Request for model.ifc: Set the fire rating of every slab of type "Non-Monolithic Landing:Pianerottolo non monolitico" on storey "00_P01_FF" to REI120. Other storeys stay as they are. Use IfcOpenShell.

First a look at what the model holds.

```python
import ifcopenshell
import ifcopenshell.util.element

model = ifcopenshell.open("model.ifc")
print(model.schema)
storey = next(s for s in model.by_type("IfcBuildingStorey") if s.Name == "00_P01_FF")
slabs = [e for e in ifcopenshell.util.element.get_decomposition(storey) if e.is_a("IfcSlab")]
seen = {}
for e in slabs:
    element_type = ifcopenshell.util.element.get_type(e)
    key = (element_type.Name if element_type != e and element_type else None, ifcopenshell.util.element.get_pset(e, "Pset_SlabCommon", "FireRating"))
    seen[key] = seen.get(key, 0) + 1
for (name, value), count in sorted(seen.items(), key=str):
    print(count, "x", name, "|", value)
```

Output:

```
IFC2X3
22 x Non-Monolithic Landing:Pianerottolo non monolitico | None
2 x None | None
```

```python
import ifcopenshell
import ifcopenshell.api.pset
import ifcopenshell.util.element

model = ifcopenshell.open("model.ifc")

storey = next(s for s in model.by_type("IfcBuildingStorey") if s.Name == "00_P01_FF")
slabs = [e for e in ifcopenshell.util.element.get_decomposition(storey) if e.is_a("IfcSlab")]

count = 0
for e in slabs:
    element_type = ifcopenshell.util.element.get_type(e)
    if element_type in (None, e) or element_type.Name != "Non-Monolithic Landing:Pianerottolo non monolitico":
        continue
    # add_pset returns the element's existing set when there is one.
    pset = ifcopenshell.api.pset.add_pset(model, product=e, name="Pset_SlabCommon")
    ifcopenshell.api.pset.edit_pset(model, pset=pset, properties={"FireRating": "REI120"})
    count += 1

print(count, "slabs updated")

model.write("model-out.ifc")
```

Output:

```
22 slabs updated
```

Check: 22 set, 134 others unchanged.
